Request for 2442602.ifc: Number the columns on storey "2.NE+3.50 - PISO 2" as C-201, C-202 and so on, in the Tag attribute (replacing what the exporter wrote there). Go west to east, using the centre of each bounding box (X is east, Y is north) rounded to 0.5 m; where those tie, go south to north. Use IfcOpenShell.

First a look at what the model holds.

```python
import ifcopenshell
import ifcopenshell.util.element
import ifcopenshell.util.placement

model = ifcopenshell.open("2442602.ifc")
print(model.schema)
storey = next(s for s in model.by_type("IfcBuildingStorey") if s.Name == "2.NE+3.50 - PISO 2")
columns = [e for e in ifcopenshell.util.element.get_decomposition(storey) if e.is_a("IfcColumn")]
for e in sorted(columns, key=lambda e: e.id()):
    origin = ifcopenshell.util.placement.get_local_placement(e.ObjectPlacement)[:3, 3]
    print(e.id(), e.Tag, e.Name, origin.round(2) + 0.0, sep=" | ")
```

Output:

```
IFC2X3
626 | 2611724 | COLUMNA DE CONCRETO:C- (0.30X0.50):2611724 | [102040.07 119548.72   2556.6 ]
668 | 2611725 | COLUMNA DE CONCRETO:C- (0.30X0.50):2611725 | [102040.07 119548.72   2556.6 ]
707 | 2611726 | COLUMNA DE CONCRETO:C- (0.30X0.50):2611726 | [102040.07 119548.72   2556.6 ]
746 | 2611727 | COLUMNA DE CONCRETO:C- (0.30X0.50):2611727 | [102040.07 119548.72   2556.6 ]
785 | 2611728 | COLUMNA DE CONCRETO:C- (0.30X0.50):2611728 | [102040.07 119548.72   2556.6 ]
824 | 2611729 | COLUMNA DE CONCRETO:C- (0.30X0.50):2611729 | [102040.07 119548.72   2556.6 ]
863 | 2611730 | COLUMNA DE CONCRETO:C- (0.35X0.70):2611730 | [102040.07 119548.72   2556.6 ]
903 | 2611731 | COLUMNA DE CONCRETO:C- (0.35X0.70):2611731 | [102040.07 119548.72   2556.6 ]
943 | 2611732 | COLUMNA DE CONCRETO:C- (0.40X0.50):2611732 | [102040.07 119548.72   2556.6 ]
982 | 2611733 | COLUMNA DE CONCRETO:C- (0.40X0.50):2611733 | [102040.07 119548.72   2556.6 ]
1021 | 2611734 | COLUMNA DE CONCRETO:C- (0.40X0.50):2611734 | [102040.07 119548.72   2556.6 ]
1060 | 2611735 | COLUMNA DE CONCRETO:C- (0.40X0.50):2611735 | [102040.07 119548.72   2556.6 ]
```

```python
import ifcopenshell
import ifcopenshell.geom
import ifcopenshell.util.element
import ifcopenshell.util.shape

model = ifcopenshell.open("2442602.ifc")
settings = ifcopenshell.geom.settings()
settings.set("use-world-coords", True)


def centre(element):
    shape = ifcopenshell.geom.create_shape(settings, element)
    return ifcopenshell.util.shape.get_bbox_centroid(shape.geometry)


storey = next(s for s in model.by_type("IfcBuildingStorey") if s.Name == "2.NE+3.50 - PISO 2")
columns = [e for e in ifcopenshell.util.element.get_decomposition(storey) if e.is_a("IfcColumn")]

# Insertion points can sit at a corner or the storey origin, so sort by the geometry (in metres).
centres = {e: centre(e) for e in columns}
columns.sort(key=lambda e: (round(centres[e][0] / 0.5), centres[e][1]))

for i, e in enumerate(columns, start=1):
    number = f"C-2{i:02d}"
    e.Tag = number
    print(e.id(), number)

model.write("2442602_rev.ifc")
```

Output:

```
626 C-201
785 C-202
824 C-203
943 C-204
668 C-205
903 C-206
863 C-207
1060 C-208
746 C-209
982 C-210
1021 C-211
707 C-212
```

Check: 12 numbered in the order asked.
